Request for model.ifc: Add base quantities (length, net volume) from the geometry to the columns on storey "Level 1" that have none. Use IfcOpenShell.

First a look at what the model holds.

```python
import ifcopenshell
import ifcopenshell.util.element
import ifcopenshell.util.unit

model = ifcopenshell.open("model.ifc")
print(model.schema)
for unit_type in ("LENGTHUNIT", "AREAUNIT", "VOLUMEUNIT"):
    print(unit_type, ifcopenshell.util.unit.calculate_unit_scale(model, unit_type))
storey = next(s for s in model.by_type("IfcBuildingStorey") if s.Name == "Level 1")
columns = [e for e in ifcopenshell.util.element.get_decomposition(storey) if e.is_a("IfcColumn")]
for e in sorted(columns, key=lambda e: e.id()):
    print(e.id(), e.is_a(), e.Name, list(ifcopenshell.util.element.get_psets(e, qtos_only=True)), sep=" | ")
```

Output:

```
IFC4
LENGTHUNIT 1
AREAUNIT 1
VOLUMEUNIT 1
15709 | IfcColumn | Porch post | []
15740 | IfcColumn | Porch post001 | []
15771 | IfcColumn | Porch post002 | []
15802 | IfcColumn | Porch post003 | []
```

```python
import ifcopenshell
import ifcopenshell.api.pset
import ifcopenshell.geom
import ifcopenshell.util.element
import ifcopenshell.util.shape
import ifcopenshell.util.unit

model = ifcopenshell.open("model.ifc")
unit_scale = ifcopenshell.util.unit.calculate_unit_scale(model)
volume_scale = ifcopenshell.util.unit.calculate_unit_scale(model, "VOLUMEUNIT")
settings = ifcopenshell.geom.settings()

storey = next(s for s in model.by_type("IfcBuildingStorey") if s.Name == "Level 1")
columns = [e for e in ifcopenshell.util.element.get_decomposition(storey) if e.is_a("IfcColumn")]

for e in sorted(columns, key=lambda e: e.id()):
    if ifcopenshell.util.element.get_psets(e, qtos_only=True, should_inherit=False):
        continue
    # Geometry comes back in metres, in the element's own axes.
    shape = ifcopenshell.geom.create_shape(settings, e)
    values = {
        "Length": ifcopenshell.util.shape.get_z(shape.geometry) / unit_scale,
        "NetVolume": ifcopenshell.util.shape.get_volume(shape.geometry) / volume_scale,
    }
    qto = ifcopenshell.api.pset.add_qto(model, product=e, name="Qto_ColumnBaseQuantities")
    ifcopenshell.api.pset.edit_qto(model, qto=qto, properties=values)
    print(e.id(), {k: round(v, 3) for k, v in values.items()})

model.write("model_v2.ifc")
```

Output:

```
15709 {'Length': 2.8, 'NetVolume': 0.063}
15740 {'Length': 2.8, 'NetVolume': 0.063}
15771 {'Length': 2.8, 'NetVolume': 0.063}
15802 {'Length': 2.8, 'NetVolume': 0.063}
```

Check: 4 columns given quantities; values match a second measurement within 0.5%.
